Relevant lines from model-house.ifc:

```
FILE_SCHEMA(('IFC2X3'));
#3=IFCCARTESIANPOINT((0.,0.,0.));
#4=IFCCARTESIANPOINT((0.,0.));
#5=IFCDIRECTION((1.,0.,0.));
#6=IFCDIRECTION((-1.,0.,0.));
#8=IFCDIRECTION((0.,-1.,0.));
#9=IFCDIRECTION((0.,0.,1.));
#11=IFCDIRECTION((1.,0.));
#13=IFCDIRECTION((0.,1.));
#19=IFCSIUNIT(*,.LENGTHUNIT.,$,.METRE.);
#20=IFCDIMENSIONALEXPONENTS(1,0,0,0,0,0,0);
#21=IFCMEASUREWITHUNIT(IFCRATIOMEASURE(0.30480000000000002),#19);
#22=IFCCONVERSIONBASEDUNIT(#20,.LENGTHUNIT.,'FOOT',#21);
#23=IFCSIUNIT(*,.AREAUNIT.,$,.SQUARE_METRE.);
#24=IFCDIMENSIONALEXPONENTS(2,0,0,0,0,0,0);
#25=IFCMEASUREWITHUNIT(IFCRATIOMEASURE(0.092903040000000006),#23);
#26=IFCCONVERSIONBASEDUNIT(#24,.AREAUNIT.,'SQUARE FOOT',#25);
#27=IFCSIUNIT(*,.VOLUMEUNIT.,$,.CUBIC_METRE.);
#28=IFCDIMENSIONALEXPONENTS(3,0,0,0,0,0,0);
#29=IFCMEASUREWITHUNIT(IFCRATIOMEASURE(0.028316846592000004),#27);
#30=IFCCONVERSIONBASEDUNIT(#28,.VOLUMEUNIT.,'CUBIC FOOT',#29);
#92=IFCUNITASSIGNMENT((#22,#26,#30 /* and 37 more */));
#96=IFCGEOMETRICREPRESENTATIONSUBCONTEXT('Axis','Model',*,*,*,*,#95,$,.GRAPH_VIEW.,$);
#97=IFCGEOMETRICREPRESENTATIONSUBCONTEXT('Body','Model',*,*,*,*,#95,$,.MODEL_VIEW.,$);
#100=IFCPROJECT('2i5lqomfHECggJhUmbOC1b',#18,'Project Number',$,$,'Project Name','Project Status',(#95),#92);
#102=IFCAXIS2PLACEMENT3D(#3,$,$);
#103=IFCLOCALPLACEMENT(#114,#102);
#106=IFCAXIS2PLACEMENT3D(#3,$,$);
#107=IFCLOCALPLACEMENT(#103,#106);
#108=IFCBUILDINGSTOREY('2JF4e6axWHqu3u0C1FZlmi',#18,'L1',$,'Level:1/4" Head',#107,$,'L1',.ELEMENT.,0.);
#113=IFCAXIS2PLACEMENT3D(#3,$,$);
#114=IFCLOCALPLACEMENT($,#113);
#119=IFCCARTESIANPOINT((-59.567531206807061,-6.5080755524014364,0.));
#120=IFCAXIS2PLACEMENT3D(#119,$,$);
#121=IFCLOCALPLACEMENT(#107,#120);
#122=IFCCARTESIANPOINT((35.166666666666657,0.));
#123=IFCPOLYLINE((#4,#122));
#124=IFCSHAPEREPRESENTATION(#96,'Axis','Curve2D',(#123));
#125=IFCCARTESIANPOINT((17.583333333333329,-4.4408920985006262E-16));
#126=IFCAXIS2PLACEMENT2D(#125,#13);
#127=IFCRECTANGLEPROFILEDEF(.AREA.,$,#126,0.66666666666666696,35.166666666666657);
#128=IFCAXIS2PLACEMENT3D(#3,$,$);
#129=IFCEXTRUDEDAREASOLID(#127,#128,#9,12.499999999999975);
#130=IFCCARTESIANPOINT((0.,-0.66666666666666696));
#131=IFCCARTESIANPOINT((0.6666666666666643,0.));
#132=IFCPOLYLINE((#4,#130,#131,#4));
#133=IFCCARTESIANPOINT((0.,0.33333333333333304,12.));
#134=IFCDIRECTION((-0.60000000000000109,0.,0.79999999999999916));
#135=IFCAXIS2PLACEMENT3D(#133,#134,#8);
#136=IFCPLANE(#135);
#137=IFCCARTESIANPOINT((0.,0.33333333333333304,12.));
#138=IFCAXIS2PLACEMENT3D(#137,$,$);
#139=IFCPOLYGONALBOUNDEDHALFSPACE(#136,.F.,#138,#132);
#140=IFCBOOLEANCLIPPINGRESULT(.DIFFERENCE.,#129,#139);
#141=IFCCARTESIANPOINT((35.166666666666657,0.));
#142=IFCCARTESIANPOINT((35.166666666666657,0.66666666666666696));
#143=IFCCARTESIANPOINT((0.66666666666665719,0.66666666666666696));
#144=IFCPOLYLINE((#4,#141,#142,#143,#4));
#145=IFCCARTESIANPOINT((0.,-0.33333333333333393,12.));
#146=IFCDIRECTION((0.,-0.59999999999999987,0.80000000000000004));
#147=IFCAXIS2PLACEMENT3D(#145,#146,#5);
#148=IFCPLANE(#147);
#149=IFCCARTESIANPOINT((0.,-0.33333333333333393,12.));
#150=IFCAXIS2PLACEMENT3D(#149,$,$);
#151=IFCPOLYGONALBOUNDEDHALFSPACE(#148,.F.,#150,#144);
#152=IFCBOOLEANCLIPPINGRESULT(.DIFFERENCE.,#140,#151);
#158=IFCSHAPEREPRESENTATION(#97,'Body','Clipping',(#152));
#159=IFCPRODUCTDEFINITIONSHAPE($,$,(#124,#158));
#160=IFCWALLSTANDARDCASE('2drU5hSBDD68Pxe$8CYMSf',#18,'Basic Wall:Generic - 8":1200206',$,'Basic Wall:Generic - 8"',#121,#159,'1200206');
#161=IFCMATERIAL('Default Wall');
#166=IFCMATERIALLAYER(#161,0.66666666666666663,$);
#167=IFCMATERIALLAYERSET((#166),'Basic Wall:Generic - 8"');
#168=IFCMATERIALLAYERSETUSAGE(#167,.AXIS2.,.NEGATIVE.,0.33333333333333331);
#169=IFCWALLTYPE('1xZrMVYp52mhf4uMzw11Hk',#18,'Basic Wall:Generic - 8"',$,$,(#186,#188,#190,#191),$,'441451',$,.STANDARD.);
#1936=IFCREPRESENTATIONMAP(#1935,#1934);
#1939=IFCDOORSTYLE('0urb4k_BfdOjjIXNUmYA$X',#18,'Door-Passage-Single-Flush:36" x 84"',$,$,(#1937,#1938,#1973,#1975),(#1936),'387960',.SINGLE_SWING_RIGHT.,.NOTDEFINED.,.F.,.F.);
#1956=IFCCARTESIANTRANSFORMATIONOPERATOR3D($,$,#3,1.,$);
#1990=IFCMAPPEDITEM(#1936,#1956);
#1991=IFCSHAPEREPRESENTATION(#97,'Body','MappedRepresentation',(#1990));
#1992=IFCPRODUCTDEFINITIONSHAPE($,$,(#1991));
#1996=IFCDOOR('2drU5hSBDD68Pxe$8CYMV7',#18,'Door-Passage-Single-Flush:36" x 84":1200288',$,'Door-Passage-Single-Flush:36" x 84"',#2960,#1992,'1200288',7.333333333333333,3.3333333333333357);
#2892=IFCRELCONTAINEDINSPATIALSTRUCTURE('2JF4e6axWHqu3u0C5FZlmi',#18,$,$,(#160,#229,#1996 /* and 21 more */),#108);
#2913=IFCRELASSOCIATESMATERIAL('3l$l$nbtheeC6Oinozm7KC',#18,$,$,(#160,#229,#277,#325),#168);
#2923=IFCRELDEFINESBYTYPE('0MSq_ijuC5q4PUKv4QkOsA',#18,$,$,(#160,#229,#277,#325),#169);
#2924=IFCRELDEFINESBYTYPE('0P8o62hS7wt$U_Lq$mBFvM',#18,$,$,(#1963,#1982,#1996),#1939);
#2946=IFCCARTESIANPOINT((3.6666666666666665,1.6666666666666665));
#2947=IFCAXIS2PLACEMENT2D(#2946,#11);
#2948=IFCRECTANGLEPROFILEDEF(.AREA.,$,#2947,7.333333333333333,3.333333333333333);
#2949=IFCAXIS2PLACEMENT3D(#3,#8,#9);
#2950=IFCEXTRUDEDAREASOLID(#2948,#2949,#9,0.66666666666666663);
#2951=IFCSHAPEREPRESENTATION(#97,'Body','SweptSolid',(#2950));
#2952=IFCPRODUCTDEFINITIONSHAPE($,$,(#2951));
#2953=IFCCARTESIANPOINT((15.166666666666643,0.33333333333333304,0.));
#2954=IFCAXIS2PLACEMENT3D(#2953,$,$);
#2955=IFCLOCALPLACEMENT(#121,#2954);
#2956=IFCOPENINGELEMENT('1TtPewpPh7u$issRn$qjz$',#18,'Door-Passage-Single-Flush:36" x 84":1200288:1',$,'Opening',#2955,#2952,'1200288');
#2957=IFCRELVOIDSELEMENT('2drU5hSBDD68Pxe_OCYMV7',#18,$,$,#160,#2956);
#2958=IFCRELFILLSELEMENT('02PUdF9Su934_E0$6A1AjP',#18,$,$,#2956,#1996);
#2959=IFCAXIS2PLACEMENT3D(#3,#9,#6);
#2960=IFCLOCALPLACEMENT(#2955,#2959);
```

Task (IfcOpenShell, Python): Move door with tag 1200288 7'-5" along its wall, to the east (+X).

```python
import ifcopenshell
import ifcopenshell.api.geometry
import ifcopenshell.util.placement
import ifcopenshell.util.unit

model = ifcopenshell.open("model-house.ifc")
unit_scale = ifcopenshell.util.unit.calculate_unit_scale(model)

door = model.by_guid("2drU5hSBDD68Pxe$8CYMV7")
opening = door.FillsVoids[0].RelatingOpeningElement
wall = opening.VoidsElements[0].RelatingBuildingElement

wall_matrix = ifcopenshell.util.placement.get_local_placement(wall.ObjectPlacement)
shift = wall_matrix[:3, 0] * 89 * 0.0254 / unit_scale
before = ifcopenshell.util.placement.get_local_placement(door.ObjectPlacement)[:3, 3].copy()

# The door is placed relative to its opening, so it follows when the opening moves.
matrix = ifcopenshell.util.placement.get_local_placement(opening.ObjectPlacement)
matrix[:3, 3] += shift
ifcopenshell.api.geometry.edit_object_placement(
    model, product=opening, matrix=matrix, is_si=False, should_transform_children=True
)

after = ifcopenshell.util.placement.get_local_placement(door.ObjectPlacement)[:3, 3]
print("door moved by", (after - before).round(3) + 0.0)

model.write("model-house_updated.ifc")
```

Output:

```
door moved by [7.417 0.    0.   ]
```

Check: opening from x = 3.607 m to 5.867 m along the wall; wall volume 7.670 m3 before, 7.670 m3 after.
